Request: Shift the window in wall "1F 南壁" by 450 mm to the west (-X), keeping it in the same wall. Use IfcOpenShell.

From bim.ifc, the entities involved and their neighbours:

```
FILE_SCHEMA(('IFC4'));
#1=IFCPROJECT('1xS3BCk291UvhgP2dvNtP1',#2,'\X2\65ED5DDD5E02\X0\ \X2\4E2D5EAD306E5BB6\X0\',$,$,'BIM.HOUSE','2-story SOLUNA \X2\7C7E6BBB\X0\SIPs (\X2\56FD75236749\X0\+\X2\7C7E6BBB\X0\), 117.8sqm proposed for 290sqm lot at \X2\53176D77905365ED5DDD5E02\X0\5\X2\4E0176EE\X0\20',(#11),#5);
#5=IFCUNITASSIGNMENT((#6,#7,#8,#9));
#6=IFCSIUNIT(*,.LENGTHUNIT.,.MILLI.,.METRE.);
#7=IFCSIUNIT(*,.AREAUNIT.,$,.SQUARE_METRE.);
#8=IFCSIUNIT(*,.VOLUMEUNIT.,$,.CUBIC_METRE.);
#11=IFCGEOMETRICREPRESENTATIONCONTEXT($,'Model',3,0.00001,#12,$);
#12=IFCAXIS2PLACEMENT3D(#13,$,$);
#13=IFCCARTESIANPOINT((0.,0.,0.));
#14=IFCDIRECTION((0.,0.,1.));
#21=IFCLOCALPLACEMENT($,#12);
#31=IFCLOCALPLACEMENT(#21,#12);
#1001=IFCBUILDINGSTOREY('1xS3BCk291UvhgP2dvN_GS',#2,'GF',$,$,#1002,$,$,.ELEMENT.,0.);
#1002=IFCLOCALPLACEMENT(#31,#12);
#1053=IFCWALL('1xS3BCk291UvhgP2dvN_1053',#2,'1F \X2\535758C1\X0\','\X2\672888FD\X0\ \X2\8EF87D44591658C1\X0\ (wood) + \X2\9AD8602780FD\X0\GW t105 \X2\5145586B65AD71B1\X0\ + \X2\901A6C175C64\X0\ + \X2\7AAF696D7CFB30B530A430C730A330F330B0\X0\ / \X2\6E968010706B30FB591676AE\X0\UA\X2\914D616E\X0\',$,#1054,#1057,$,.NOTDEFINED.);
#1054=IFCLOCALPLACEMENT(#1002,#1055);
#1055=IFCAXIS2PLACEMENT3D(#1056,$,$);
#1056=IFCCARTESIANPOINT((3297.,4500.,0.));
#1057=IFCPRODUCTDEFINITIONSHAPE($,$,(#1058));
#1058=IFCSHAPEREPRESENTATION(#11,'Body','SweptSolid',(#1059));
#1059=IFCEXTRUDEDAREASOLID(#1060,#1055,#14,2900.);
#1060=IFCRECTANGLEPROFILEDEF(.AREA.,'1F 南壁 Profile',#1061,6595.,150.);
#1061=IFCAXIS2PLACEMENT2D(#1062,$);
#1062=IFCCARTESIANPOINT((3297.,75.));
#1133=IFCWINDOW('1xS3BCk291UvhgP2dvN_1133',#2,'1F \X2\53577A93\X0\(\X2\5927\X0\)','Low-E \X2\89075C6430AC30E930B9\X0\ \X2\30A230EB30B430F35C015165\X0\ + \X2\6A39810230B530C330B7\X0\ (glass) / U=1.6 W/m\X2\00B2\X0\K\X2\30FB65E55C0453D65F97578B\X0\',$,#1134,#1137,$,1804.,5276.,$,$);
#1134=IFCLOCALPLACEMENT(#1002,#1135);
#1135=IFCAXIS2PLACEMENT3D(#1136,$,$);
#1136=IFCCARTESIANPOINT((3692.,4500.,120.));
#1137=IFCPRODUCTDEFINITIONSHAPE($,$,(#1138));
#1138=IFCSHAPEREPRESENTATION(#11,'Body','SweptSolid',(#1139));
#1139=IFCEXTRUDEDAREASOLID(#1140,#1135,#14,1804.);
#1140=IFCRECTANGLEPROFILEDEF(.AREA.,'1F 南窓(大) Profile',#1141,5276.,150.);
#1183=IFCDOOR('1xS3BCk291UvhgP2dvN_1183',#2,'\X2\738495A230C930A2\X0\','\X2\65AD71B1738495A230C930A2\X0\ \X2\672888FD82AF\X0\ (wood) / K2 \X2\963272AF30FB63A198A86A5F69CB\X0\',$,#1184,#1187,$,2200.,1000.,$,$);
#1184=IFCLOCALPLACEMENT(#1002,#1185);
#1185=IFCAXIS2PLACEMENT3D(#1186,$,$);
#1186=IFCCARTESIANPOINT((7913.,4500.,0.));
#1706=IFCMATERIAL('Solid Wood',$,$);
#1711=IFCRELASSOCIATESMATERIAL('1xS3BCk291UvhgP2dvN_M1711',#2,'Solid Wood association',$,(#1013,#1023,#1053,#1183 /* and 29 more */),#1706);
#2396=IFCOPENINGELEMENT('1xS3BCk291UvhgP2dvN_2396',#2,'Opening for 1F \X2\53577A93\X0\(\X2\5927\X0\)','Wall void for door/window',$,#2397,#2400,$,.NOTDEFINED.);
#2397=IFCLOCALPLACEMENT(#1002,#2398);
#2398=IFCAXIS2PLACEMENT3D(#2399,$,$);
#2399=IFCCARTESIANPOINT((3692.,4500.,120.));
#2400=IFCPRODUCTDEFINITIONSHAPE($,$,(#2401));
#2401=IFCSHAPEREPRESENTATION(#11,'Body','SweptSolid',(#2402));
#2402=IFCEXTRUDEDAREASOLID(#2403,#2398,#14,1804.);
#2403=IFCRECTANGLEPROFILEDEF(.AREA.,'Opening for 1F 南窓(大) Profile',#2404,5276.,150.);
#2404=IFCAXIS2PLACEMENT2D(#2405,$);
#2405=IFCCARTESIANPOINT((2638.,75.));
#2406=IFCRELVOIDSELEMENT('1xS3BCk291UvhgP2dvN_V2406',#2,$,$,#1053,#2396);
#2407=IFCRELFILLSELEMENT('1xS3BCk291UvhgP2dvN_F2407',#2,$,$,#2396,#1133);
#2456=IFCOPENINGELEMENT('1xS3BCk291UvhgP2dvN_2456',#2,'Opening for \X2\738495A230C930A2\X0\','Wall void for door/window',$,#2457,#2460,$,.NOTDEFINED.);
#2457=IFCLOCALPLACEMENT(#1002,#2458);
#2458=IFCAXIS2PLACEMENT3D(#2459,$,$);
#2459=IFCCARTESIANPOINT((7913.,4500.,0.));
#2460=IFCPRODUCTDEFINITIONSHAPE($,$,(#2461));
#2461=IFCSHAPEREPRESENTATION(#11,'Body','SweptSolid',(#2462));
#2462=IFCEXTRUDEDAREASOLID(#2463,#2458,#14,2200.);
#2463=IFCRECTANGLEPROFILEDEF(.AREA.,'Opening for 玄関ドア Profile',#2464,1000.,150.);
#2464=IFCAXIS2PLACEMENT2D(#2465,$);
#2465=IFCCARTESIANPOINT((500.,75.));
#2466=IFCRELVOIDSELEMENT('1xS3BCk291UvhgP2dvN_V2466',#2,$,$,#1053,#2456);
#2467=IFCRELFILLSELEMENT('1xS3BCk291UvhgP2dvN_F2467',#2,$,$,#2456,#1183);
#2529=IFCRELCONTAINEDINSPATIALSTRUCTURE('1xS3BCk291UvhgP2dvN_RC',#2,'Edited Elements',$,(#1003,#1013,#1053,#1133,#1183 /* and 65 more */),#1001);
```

```python
import ifcopenshell
import ifcopenshell.api.geometry
import ifcopenshell.util.placement
import ifcopenshell.util.unit

model = ifcopenshell.open("bim.ifc")
unit_scale = ifcopenshell.util.unit.calculate_unit_scale(model)

window = model.by_guid("1xS3BCk291UvhgP2dvN_1133")
opening = window.FillsVoids[0].RelatingOpeningElement
wall = opening.VoidsElements[0].RelatingBuildingElement

wall_matrix = ifcopenshell.util.placement.get_local_placement(wall.ObjectPlacement)
shift = wall_matrix[:3, 0] * -0.45 / unit_scale
before = ifcopenshell.util.placement.get_local_placement(window.ObjectPlacement)[:3, 3].copy()

# The window is not placed relative to its opening, so move both.
for product in (opening, window):
    matrix = ifcopenshell.util.placement.get_local_placement(product.ObjectPlacement)
    matrix[:3, 3] += shift
    ifcopenshell.api.geometry.edit_object_placement(model, product=product, matrix=matrix, is_si=False)

after = ifcopenshell.util.placement.get_local_placement(window.ObjectPlacement)[:3, 3]
print("window moved by", (after - before).round(3) + 0.0)

model.write("bim_updated.ifc")
```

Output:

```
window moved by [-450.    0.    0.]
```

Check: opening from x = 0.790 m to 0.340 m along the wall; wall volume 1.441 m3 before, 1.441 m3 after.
